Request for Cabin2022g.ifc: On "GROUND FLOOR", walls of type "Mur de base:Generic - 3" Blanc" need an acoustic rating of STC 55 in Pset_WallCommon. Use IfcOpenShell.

First a look at what the model holds.

```python
import ifcopenshell
import ifcopenshell.util.element

model = ifcopenshell.open("Cabin2022g.ifc")
print(model.schema)
storey = next(s for s in model.by_type("IfcBuildingStorey") if s.Name == "GROUND FLOOR")
walls = [e for e in ifcopenshell.util.element.get_decomposition(storey) if e.is_a("IfcWall")]
seen = {}
for e in walls:
    element_type = ifcopenshell.util.element.get_type(e)
    key = (element_type.Name if element_type != e and element_type else None, ifcopenshell.util.element.get_pset(e, "Pset_WallCommon", "AcousticRating"))
    seen[key] = seen.get(key, 0) + 1
for (name, value), count in sorted(seen.items(), key=str):
    print(count, "x", name, "|", value)
```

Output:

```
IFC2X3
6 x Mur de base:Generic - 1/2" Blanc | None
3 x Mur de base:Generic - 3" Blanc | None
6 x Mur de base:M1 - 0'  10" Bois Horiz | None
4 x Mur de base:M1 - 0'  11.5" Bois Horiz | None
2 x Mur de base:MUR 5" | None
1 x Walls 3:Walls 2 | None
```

```python
import ifcopenshell
import ifcopenshell.api.pset
import ifcopenshell.util.element

model = ifcopenshell.open("Cabin2022g.ifc")

storey = next(s for s in model.by_type("IfcBuildingStorey") if s.Name == "GROUND FLOOR")
walls = [e for e in ifcopenshell.util.element.get_decomposition(storey) if e.is_a("IfcWall")]

count = 0
for e in walls:
    element_type = ifcopenshell.util.element.get_type(e)
    if element_type in (None, e) or element_type.Name != 'Mur de base:Generic - 3" Blanc':
        continue
    # add_pset returns the element's existing set when there is one.
    pset = ifcopenshell.api.pset.add_pset(model, product=e, name="Pset_WallCommon")
    ifcopenshell.api.pset.edit_pset(model, pset=pset, properties={"AcousticRating": "STC 55"})
    count += 1

print(count, "walls updated")

model.write("Cabin2022g_updated.ifc")
```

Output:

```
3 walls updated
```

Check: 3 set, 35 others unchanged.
